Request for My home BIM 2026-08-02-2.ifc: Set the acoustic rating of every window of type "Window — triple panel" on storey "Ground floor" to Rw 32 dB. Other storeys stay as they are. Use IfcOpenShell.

First a look at what the model holds.

```python
import ifcopenshell
import ifcopenshell.util.element

model = ifcopenshell.open("My home BIM 2026-08-02-2.ifc")
print(model.schema)
storey = next(s for s in model.by_type("IfcBuildingStorey") if s.Name == "Ground floor")
windows = [e for e in ifcopenshell.util.element.get_decomposition(storey) if e.is_a("IfcWindow")]
seen = {}
for e in windows:
    element_type = ifcopenshell.util.element.get_type(e)
    key = (element_type.Name if element_type != e and element_type else None, ifcopenshell.util.element.get_pset(e, "Pset_WindowCommon", "AcousticRating"))
    seen[key] = seen.get(key, 0) + 1
for (name, value), count in sorted(seen.items(), key=str):
    print(count, "x", name, "|", value)
```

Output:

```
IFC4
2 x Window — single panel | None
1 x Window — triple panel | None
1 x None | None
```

```python
import ifcopenshell
import ifcopenshell.api.pset
import ifcopenshell.util.element

model = ifcopenshell.open("My home BIM 2026-08-02-2.ifc")

storey = next(s for s in model.by_type("IfcBuildingStorey") if s.Name == "Ground floor")
windows = [e for e in ifcopenshell.util.element.get_decomposition(storey) if e.is_a("IfcWindow")]

count = 0
for e in windows:
    element_type = ifcopenshell.util.element.get_type(e)
    if element_type in (None, e) or element_type.Name != "Window — triple panel":
        continue
    # add_pset returns the element's existing set when there is one.
    pset = ifcopenshell.api.pset.add_pset(model, product=e, name="Pset_WindowCommon")
    ifcopenshell.api.pset.edit_pset(model, pset=pset, properties={"AcousticRating": "Rw 32 dB"})
    count += 1

print(count, "windows updated")

model.write("My home BIM 2026-08-02-2_v2.ifc")
```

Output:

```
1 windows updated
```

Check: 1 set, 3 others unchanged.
